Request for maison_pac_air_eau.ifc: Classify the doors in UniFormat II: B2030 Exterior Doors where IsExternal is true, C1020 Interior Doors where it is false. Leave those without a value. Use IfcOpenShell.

First a look at what the model holds.

```python
import ifcopenshell
import ifcopenshell.util.element

model = ifcopenshell.open("maison_pac_air_eau.ifc")
print(model.schema)
print("classifications:", [c.Name for c in model.by_type("IfcClassification")])
values = [ifcopenshell.util.element.get_pset(e, "Pset_DoorCommon", "IsExternal") for e in model.by_type("IfcDoor")]
for value in (True, False, None):
    print("IsExternal", value, values.count(value))
```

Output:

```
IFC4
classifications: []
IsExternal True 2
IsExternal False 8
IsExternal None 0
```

```python
import ifcopenshell
import ifcopenshell.api.classification
import ifcopenshell.util.element

model = ifcopenshell.open("maison_pac_air_eau.ifc")

system = ifcopenshell.api.classification.add_classification(model, classification="UniFormat II")

doors = model.by_type("IfcDoor")
external = {e: ifcopenshell.util.element.get_pset(e, "Pset_DoorCommon", "IsExternal") for e in doors}
for flag, code, name in ((True, "B2030", "Exterior Doors"), (False, "C1020", "Interior Doors")):
    products = [e for e in doors if external[e] is flag]
    ifcopenshell.api.classification.add_reference(
        model, products=products, classification=system, identification=code, name=name
    )
    print(code, len(products))

model.write("maison_pac_air_eau_updated.ifc")
```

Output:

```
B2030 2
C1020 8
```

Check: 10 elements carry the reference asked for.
